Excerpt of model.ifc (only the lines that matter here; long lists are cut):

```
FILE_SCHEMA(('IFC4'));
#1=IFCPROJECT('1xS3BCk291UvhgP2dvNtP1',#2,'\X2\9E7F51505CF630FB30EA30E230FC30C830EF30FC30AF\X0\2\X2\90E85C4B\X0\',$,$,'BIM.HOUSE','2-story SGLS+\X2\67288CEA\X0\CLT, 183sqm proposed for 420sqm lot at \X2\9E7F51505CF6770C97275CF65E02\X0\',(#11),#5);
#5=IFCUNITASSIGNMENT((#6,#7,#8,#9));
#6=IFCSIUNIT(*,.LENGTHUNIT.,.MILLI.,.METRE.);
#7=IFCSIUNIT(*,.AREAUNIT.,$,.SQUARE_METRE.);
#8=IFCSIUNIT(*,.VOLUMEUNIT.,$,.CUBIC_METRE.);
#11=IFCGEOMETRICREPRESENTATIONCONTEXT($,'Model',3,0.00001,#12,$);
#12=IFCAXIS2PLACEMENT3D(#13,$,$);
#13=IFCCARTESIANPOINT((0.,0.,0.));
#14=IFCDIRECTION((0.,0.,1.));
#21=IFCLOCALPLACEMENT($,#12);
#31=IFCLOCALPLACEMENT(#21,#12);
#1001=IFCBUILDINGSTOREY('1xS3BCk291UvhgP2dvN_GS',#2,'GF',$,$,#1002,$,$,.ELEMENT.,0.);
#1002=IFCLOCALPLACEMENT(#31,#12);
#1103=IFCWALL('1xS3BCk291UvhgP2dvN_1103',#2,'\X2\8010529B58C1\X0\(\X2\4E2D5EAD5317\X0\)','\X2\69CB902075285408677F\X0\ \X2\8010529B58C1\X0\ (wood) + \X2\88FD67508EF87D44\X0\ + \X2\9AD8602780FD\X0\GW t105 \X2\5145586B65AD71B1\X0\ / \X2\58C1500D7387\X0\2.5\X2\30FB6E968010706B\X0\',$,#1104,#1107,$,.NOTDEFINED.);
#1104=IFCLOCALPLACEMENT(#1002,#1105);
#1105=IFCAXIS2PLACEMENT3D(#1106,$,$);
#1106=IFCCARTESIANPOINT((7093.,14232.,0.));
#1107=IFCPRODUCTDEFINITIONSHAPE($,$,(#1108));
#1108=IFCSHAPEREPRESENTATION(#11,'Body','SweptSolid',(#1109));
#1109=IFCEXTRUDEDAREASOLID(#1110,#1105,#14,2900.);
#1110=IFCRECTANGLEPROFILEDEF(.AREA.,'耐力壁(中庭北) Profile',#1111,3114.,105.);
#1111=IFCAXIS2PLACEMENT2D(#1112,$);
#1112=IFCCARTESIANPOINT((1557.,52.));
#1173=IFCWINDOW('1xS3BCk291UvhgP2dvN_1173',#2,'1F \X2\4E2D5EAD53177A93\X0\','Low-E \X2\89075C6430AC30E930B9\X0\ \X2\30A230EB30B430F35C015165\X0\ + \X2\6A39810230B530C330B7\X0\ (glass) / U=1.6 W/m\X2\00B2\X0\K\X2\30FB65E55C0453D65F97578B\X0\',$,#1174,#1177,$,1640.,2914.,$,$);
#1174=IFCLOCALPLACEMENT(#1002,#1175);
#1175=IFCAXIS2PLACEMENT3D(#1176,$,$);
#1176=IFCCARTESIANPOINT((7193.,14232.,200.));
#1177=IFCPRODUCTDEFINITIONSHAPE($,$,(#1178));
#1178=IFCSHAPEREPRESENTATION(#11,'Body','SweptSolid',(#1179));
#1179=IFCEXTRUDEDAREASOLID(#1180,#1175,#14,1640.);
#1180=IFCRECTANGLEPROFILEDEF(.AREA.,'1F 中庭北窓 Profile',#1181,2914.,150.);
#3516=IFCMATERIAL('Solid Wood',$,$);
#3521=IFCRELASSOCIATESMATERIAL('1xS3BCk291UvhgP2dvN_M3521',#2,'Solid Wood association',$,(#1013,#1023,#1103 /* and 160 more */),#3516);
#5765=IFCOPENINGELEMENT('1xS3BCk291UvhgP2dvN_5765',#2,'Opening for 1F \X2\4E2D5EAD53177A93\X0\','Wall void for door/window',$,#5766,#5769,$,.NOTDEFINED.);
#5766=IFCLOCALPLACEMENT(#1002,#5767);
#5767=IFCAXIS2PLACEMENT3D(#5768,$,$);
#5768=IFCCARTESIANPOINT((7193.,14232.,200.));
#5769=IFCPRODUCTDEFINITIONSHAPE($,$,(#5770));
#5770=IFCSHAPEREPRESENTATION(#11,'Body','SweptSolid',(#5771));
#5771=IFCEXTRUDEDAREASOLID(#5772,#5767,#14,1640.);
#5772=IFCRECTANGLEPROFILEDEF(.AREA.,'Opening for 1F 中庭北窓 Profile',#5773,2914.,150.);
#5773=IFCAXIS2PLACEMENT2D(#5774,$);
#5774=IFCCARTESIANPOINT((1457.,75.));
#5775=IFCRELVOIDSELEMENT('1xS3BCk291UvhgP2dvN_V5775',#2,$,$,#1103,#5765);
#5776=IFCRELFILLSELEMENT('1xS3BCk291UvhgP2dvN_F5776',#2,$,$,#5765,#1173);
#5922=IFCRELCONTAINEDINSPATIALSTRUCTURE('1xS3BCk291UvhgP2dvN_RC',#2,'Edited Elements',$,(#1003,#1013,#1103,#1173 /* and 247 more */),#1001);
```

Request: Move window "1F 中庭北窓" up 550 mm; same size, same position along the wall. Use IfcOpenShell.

```python
import numpy as np
import ifcopenshell
import ifcopenshell.api.geometry
import ifcopenshell.util.placement
import ifcopenshell.util.unit

model = ifcopenshell.open("model.ifc")
unit_scale = ifcopenshell.util.unit.calculate_unit_scale(model)

window = model.by_guid("1xS3BCk291UvhgP2dvN_1173")
opening = window.FillsVoids[0].RelatingOpeningElement
dz = 550.0

shift = np.array([0.0, 0.0, dz])
# The window is not placed relative to its opening, so move both.
for product in (opening, window):
    matrix = ifcopenshell.util.placement.get_local_placement(product.ObjectPlacement)
    matrix[:3, 3] += shift
    ifcopenshell.api.geometry.edit_object_placement(model, product=product, matrix=matrix, is_si=False)

print(f"moved by {dz * unit_scale:+.3f} m")

model.write("model_v2.ifc")
```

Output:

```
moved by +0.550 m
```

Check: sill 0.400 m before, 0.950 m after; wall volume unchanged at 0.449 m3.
